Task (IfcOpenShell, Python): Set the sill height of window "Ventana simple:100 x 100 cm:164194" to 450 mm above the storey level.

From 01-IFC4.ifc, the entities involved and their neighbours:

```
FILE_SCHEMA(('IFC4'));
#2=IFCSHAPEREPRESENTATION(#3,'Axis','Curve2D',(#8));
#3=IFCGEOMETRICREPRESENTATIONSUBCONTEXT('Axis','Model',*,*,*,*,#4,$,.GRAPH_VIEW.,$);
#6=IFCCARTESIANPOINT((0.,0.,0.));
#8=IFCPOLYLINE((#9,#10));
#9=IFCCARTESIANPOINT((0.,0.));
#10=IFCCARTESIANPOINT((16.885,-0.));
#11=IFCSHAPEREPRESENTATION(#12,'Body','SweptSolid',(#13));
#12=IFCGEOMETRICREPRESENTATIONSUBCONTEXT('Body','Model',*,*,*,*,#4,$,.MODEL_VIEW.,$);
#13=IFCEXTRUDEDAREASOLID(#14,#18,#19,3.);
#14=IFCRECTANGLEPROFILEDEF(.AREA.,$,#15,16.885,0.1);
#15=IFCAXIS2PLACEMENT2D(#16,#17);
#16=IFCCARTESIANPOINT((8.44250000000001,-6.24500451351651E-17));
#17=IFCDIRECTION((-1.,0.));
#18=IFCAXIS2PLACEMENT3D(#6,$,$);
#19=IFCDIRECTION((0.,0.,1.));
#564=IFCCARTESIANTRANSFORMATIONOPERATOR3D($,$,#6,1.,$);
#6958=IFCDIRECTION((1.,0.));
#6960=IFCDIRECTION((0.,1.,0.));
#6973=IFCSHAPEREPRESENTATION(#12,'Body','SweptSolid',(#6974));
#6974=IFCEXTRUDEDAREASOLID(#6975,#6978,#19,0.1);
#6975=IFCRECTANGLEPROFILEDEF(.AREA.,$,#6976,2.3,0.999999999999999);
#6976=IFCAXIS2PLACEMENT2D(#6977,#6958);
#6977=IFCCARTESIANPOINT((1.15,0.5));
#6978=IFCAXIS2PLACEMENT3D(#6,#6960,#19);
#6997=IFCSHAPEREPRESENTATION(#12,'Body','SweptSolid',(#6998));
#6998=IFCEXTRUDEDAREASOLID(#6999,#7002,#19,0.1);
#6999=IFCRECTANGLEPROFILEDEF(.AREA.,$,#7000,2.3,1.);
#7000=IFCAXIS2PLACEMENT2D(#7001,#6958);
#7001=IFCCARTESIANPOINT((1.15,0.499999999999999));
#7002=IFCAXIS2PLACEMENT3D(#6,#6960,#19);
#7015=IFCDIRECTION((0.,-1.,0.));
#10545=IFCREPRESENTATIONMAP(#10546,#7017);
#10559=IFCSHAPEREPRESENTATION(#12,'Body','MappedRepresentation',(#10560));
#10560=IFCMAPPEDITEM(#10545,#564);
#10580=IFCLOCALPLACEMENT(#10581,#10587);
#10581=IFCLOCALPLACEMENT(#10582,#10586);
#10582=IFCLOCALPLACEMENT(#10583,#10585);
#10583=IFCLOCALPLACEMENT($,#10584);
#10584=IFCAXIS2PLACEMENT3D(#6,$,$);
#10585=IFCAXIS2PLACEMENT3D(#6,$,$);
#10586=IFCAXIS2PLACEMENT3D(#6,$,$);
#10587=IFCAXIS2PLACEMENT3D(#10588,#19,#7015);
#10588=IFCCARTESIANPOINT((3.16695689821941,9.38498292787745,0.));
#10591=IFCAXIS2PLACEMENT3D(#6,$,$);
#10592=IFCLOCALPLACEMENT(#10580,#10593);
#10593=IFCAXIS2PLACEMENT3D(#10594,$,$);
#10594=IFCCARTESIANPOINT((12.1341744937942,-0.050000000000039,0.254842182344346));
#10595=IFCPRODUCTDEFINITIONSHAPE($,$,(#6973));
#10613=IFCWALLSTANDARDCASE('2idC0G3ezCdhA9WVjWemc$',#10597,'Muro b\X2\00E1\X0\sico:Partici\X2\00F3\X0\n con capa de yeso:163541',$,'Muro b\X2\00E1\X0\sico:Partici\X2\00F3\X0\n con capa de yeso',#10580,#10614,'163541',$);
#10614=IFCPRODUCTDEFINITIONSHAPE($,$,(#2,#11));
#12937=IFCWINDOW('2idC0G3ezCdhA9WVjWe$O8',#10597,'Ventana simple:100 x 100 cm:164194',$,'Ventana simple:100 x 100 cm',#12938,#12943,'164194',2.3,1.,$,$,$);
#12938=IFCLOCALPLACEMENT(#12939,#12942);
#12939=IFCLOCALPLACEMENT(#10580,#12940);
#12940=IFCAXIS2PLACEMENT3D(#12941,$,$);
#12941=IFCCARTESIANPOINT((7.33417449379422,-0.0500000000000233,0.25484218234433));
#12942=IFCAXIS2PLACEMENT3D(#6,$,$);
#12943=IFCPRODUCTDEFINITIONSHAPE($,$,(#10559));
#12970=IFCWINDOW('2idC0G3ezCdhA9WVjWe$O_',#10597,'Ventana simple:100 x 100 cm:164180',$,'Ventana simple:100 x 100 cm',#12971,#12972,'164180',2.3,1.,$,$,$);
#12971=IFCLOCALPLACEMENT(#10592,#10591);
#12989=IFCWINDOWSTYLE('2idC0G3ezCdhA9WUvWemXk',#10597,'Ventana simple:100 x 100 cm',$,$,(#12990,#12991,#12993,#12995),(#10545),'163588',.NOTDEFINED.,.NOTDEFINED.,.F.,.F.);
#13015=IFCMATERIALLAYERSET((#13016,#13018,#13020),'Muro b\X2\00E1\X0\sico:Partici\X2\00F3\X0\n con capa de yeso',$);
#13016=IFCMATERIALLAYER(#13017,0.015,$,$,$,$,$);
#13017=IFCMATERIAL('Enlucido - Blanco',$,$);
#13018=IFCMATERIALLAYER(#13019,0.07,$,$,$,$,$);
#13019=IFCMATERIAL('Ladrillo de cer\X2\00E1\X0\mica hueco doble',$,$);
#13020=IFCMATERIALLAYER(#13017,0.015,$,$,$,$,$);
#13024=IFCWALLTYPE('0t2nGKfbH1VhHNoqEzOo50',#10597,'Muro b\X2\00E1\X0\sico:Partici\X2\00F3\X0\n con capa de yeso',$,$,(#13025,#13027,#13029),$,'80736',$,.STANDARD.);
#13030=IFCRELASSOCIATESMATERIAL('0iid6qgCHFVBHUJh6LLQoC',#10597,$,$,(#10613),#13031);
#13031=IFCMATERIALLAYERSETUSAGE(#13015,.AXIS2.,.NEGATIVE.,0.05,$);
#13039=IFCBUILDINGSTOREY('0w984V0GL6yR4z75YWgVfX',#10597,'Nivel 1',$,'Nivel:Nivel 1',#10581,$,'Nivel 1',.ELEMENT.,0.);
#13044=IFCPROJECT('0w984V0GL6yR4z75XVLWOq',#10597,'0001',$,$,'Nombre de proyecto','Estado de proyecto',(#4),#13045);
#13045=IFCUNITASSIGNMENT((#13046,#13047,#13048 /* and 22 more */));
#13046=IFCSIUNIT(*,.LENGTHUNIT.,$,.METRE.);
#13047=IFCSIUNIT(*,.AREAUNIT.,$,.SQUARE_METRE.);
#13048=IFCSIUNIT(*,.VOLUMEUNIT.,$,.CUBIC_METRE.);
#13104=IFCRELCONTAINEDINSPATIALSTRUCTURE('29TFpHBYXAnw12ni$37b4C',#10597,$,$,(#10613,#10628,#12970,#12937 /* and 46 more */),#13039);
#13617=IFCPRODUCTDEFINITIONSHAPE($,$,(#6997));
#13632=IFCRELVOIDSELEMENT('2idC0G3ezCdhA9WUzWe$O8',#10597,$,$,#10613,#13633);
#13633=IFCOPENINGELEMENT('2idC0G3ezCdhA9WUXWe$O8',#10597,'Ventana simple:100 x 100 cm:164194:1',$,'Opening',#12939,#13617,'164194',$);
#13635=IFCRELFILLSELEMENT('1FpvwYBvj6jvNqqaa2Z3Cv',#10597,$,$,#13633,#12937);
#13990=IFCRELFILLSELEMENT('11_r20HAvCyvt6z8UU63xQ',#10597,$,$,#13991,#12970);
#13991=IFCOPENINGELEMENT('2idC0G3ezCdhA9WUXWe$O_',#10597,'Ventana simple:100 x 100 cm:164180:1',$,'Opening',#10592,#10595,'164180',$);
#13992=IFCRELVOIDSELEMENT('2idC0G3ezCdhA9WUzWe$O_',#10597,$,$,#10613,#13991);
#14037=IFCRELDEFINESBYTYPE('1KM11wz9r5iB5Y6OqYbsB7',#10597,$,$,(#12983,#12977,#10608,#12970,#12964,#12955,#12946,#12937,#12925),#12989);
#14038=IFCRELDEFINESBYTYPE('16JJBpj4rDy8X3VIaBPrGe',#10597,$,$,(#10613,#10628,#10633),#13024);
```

```python
import numpy as np
import ifcopenshell
import ifcopenshell.api.geometry
import ifcopenshell.geom
import ifcopenshell.util.element
import ifcopenshell.util.placement
import ifcopenshell.util.shape
import ifcopenshell.util.unit

model = ifcopenshell.open("01-IFC4.ifc")
unit_scale = ifcopenshell.util.unit.calculate_unit_scale(model)

window = model.by_guid("2idC0G3ezCdhA9WVjWe$O8")
opening = window.FillsVoids[0].RelatingOpeningElement
storey = ifcopenshell.util.element.get_container(window, ifc_class="IfcBuildingStorey")
level = ifcopenshell.util.placement.get_local_placement(storey.ObjectPlacement)[2, 3]

# The opening's origin need not be at the sill, so measure its lowest point.
shape = ifcopenshell.geom.create_shape(ifcopenshell.geom.settings(), opening)
bottom = ifcopenshell.util.shape.get_shape_bottom_elevation(shape, shape.geometry) / unit_scale
dz = level + 0.45 - bottom

shift = np.array([0.0, 0.0, dz])
# The window is placed relative to its opening, so it follows when the opening moves.
matrix = ifcopenshell.util.placement.get_local_placement(opening.ObjectPlacement)
matrix[:3, 3] += shift
ifcopenshell.api.geometry.edit_object_placement(
    model, product=opening, matrix=matrix, is_si=False, should_transform_children=True
)

print(f"moved by {dz * unit_scale:+.3f} m")

model.write("01-IFC4-out.ifc")
```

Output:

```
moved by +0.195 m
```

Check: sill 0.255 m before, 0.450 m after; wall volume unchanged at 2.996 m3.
